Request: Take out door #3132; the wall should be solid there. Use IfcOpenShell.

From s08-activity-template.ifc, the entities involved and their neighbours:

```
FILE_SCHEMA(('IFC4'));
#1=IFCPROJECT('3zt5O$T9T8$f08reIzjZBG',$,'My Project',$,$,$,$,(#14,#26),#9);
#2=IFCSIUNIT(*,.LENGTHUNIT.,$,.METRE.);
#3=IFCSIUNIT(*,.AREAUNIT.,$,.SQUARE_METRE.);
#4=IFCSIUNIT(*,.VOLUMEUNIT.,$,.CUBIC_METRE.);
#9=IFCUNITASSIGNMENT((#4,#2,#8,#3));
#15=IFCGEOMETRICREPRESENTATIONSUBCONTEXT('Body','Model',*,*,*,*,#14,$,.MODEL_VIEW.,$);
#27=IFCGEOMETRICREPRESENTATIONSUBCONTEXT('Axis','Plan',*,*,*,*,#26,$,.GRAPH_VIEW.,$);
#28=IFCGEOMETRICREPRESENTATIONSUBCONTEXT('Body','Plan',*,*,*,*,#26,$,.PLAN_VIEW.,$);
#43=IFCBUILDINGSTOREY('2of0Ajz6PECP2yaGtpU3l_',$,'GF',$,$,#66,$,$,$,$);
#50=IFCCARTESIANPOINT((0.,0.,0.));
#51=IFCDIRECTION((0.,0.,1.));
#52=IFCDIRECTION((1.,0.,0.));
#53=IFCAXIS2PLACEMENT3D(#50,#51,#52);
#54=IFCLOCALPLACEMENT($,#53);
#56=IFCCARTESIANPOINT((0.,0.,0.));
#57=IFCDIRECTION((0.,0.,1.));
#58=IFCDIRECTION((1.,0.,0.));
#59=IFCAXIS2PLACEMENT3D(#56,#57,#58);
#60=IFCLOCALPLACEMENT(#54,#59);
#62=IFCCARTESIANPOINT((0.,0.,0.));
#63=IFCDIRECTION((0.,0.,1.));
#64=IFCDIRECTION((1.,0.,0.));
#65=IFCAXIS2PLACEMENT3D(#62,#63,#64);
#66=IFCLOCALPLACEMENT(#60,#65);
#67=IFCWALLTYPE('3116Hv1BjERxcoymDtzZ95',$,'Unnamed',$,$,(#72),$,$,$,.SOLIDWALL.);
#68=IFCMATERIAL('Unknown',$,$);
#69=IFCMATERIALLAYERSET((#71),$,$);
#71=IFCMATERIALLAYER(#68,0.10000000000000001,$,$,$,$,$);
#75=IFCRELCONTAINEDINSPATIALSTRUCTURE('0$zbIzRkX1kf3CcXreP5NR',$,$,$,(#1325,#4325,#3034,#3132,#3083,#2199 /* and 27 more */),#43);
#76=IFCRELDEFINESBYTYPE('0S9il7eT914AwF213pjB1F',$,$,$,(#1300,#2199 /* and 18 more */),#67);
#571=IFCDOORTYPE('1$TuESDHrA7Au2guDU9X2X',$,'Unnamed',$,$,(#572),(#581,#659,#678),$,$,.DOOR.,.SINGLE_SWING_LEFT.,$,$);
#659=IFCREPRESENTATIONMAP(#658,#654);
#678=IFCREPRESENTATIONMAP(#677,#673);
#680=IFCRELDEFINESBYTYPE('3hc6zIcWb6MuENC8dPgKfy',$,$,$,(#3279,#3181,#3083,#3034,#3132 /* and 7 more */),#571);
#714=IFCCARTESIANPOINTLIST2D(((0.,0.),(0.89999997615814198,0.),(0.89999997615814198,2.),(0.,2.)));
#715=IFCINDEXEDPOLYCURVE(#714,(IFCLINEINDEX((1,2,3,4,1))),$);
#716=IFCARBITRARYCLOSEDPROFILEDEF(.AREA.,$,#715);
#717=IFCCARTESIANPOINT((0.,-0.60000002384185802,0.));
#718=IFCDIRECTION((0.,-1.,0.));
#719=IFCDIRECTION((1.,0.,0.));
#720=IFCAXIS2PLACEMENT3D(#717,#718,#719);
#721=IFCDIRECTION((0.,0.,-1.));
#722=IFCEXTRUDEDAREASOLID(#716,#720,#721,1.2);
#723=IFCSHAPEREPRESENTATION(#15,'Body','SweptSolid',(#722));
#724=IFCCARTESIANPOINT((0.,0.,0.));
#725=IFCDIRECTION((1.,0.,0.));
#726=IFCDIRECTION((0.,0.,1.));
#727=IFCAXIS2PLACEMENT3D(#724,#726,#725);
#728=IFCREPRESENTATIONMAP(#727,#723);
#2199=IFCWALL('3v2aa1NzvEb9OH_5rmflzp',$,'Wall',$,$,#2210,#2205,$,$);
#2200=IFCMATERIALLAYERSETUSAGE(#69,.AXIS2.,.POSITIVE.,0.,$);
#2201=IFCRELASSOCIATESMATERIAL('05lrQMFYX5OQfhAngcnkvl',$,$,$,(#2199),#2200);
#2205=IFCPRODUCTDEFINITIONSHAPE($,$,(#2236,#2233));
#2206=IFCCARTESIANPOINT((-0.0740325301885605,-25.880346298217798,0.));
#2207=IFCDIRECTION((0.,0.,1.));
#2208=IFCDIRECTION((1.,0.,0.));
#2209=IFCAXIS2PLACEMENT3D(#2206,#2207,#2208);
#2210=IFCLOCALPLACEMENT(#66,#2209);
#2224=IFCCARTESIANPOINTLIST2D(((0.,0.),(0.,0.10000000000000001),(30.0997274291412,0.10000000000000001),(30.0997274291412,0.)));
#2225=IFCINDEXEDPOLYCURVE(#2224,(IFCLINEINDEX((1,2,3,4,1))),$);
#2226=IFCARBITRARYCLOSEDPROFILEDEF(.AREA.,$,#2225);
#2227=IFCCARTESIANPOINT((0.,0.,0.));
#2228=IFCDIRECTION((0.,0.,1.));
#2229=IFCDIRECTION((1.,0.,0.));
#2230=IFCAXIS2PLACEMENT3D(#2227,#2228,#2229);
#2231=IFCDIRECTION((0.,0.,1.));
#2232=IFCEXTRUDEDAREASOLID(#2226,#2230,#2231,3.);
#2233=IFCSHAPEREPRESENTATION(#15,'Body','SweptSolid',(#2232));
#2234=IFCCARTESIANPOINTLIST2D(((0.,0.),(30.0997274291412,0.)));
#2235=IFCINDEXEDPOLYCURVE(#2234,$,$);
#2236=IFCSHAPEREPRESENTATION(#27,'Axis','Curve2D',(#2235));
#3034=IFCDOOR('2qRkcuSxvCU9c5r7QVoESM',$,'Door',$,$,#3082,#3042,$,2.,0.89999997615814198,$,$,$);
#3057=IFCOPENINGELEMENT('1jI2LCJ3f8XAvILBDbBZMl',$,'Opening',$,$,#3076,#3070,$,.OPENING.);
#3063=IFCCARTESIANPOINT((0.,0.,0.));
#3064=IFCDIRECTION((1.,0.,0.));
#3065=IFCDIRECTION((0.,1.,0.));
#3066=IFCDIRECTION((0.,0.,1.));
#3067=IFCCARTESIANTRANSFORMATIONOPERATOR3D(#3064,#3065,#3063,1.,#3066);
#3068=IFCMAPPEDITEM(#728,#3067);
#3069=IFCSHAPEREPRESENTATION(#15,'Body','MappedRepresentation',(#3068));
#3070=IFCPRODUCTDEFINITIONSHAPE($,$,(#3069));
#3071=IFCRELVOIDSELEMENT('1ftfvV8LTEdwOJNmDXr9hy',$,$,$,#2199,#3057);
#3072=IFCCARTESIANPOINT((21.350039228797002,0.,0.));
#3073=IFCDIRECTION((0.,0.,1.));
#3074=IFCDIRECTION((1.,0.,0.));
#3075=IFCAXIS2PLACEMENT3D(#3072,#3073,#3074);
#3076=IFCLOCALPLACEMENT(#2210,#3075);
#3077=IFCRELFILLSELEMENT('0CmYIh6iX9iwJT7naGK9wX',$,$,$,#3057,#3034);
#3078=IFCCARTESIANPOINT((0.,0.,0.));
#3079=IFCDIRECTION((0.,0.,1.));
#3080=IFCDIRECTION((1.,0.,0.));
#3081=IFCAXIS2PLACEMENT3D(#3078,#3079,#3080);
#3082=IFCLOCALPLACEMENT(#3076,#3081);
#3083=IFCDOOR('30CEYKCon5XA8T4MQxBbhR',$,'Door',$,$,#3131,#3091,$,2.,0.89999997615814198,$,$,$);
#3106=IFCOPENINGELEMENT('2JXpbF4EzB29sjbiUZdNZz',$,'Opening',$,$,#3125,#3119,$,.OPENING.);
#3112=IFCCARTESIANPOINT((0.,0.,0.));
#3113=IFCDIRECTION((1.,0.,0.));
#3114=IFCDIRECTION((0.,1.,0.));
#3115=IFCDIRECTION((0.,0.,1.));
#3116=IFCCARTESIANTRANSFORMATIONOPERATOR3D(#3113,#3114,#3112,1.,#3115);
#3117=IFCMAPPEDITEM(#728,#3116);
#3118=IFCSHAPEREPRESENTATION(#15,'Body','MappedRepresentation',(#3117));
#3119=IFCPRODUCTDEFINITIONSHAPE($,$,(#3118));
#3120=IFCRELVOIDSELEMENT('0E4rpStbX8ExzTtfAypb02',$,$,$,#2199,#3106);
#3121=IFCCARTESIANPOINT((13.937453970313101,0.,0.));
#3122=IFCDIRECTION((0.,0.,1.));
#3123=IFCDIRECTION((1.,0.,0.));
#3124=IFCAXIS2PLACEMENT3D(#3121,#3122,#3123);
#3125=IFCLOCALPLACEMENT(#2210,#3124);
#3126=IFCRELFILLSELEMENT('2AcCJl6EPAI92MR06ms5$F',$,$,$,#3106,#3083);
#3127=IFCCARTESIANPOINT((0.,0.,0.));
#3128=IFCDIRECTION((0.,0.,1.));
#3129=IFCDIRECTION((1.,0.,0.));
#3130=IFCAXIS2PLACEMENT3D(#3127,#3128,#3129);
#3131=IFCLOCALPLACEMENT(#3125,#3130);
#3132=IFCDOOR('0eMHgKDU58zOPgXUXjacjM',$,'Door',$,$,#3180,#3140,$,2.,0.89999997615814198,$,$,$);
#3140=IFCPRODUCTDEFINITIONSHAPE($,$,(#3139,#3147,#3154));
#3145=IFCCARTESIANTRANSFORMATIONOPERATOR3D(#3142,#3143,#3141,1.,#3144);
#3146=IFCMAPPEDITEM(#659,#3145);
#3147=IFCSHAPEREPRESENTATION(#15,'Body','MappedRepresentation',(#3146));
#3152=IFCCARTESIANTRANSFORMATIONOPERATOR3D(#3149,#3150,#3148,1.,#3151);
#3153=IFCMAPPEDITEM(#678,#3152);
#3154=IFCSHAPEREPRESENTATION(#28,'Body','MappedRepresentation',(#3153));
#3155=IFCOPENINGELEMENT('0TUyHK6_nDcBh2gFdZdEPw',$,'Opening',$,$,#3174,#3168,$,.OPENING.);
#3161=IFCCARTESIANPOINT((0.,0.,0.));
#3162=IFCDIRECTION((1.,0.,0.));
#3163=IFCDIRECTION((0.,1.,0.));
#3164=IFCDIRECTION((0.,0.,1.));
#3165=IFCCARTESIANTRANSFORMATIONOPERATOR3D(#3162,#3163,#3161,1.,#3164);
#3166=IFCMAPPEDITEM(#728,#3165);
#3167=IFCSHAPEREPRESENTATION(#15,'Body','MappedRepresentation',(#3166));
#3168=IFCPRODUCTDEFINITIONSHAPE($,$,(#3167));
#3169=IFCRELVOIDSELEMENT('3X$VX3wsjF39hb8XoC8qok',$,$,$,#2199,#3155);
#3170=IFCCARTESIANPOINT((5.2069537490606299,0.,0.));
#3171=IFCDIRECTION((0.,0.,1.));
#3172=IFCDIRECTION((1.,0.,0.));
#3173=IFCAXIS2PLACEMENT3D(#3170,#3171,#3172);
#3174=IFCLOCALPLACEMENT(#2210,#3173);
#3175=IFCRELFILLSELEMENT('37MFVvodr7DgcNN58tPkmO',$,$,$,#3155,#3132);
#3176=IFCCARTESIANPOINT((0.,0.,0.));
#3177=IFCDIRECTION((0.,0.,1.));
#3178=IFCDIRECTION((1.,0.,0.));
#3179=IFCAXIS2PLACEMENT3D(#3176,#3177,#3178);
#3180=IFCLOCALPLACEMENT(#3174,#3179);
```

```python
import ifcopenshell
import ifcopenshell.api.feature
import ifcopenshell.api.root
import ifcopenshell.geom
import ifcopenshell.util.shape

model = ifcopenshell.open("s08-activity-template.ifc")
settings = ifcopenshell.geom.settings()


def volume(element):
    """Net volume in cubic metres, openings subtracted."""
    shape = ifcopenshell.geom.create_shape(settings, element)
    return ifcopenshell.util.shape.get_volume(shape.geometry)


door = model.by_id(3132)
opening = door.FillsVoids[0].RelatingOpeningElement
wall = opening.VoidsElements[0].RelatingBuildingElement
before = volume(wall)

ifcopenshell.api.root.remove_product(model, product=door)
ifcopenshell.api.feature.remove_feature(model, feature=opening)

after = volume(wall)

print(f"wall volume {before:.3f} -> {after:.3f} m3")

model.write("s08-activity-template_v2.ifc")
```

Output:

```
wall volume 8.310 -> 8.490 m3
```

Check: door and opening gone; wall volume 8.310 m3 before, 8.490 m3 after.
